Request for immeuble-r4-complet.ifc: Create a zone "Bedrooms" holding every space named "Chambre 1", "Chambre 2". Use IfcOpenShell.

First a look at what the model holds.

```python
import ifcopenshell

model = ifcopenshell.open("immeuble-r4-complet.ifc")
print(model.schema)
seen = {}
for space in model.by_type("IfcSpace"):
    seen[space.Name] = seen.get(space.Name, 0) + 1
for name, count in sorted(seen.items(), key=str):
    print(count, "x", name)
print("zones:", [z.Name for z in model.by_type("IfcZone")][:20])
```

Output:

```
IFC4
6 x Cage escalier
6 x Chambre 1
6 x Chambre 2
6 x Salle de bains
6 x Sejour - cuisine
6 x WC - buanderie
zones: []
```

```python
import ifcopenshell
import ifcopenshell.api.group
import ifcopenshell.api.root

model = ifcopenshell.open("immeuble-r4-complet.ifc")

names = {"Chambre 1", "Chambre 2"}
spaces = [s for s in model.by_type("IfcSpace") if s.Name in names]

zone = ifcopenshell.api.root.create_entity(model, ifc_class="IfcZone", name="Bedrooms")
ifcopenshell.api.group.assign_group(model, products=spaces, group=zone)
print(len(spaces), "spaces in", zone.Name)

model.write("immeuble-r4-complet_rev.ifc")
```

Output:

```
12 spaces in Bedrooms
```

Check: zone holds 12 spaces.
